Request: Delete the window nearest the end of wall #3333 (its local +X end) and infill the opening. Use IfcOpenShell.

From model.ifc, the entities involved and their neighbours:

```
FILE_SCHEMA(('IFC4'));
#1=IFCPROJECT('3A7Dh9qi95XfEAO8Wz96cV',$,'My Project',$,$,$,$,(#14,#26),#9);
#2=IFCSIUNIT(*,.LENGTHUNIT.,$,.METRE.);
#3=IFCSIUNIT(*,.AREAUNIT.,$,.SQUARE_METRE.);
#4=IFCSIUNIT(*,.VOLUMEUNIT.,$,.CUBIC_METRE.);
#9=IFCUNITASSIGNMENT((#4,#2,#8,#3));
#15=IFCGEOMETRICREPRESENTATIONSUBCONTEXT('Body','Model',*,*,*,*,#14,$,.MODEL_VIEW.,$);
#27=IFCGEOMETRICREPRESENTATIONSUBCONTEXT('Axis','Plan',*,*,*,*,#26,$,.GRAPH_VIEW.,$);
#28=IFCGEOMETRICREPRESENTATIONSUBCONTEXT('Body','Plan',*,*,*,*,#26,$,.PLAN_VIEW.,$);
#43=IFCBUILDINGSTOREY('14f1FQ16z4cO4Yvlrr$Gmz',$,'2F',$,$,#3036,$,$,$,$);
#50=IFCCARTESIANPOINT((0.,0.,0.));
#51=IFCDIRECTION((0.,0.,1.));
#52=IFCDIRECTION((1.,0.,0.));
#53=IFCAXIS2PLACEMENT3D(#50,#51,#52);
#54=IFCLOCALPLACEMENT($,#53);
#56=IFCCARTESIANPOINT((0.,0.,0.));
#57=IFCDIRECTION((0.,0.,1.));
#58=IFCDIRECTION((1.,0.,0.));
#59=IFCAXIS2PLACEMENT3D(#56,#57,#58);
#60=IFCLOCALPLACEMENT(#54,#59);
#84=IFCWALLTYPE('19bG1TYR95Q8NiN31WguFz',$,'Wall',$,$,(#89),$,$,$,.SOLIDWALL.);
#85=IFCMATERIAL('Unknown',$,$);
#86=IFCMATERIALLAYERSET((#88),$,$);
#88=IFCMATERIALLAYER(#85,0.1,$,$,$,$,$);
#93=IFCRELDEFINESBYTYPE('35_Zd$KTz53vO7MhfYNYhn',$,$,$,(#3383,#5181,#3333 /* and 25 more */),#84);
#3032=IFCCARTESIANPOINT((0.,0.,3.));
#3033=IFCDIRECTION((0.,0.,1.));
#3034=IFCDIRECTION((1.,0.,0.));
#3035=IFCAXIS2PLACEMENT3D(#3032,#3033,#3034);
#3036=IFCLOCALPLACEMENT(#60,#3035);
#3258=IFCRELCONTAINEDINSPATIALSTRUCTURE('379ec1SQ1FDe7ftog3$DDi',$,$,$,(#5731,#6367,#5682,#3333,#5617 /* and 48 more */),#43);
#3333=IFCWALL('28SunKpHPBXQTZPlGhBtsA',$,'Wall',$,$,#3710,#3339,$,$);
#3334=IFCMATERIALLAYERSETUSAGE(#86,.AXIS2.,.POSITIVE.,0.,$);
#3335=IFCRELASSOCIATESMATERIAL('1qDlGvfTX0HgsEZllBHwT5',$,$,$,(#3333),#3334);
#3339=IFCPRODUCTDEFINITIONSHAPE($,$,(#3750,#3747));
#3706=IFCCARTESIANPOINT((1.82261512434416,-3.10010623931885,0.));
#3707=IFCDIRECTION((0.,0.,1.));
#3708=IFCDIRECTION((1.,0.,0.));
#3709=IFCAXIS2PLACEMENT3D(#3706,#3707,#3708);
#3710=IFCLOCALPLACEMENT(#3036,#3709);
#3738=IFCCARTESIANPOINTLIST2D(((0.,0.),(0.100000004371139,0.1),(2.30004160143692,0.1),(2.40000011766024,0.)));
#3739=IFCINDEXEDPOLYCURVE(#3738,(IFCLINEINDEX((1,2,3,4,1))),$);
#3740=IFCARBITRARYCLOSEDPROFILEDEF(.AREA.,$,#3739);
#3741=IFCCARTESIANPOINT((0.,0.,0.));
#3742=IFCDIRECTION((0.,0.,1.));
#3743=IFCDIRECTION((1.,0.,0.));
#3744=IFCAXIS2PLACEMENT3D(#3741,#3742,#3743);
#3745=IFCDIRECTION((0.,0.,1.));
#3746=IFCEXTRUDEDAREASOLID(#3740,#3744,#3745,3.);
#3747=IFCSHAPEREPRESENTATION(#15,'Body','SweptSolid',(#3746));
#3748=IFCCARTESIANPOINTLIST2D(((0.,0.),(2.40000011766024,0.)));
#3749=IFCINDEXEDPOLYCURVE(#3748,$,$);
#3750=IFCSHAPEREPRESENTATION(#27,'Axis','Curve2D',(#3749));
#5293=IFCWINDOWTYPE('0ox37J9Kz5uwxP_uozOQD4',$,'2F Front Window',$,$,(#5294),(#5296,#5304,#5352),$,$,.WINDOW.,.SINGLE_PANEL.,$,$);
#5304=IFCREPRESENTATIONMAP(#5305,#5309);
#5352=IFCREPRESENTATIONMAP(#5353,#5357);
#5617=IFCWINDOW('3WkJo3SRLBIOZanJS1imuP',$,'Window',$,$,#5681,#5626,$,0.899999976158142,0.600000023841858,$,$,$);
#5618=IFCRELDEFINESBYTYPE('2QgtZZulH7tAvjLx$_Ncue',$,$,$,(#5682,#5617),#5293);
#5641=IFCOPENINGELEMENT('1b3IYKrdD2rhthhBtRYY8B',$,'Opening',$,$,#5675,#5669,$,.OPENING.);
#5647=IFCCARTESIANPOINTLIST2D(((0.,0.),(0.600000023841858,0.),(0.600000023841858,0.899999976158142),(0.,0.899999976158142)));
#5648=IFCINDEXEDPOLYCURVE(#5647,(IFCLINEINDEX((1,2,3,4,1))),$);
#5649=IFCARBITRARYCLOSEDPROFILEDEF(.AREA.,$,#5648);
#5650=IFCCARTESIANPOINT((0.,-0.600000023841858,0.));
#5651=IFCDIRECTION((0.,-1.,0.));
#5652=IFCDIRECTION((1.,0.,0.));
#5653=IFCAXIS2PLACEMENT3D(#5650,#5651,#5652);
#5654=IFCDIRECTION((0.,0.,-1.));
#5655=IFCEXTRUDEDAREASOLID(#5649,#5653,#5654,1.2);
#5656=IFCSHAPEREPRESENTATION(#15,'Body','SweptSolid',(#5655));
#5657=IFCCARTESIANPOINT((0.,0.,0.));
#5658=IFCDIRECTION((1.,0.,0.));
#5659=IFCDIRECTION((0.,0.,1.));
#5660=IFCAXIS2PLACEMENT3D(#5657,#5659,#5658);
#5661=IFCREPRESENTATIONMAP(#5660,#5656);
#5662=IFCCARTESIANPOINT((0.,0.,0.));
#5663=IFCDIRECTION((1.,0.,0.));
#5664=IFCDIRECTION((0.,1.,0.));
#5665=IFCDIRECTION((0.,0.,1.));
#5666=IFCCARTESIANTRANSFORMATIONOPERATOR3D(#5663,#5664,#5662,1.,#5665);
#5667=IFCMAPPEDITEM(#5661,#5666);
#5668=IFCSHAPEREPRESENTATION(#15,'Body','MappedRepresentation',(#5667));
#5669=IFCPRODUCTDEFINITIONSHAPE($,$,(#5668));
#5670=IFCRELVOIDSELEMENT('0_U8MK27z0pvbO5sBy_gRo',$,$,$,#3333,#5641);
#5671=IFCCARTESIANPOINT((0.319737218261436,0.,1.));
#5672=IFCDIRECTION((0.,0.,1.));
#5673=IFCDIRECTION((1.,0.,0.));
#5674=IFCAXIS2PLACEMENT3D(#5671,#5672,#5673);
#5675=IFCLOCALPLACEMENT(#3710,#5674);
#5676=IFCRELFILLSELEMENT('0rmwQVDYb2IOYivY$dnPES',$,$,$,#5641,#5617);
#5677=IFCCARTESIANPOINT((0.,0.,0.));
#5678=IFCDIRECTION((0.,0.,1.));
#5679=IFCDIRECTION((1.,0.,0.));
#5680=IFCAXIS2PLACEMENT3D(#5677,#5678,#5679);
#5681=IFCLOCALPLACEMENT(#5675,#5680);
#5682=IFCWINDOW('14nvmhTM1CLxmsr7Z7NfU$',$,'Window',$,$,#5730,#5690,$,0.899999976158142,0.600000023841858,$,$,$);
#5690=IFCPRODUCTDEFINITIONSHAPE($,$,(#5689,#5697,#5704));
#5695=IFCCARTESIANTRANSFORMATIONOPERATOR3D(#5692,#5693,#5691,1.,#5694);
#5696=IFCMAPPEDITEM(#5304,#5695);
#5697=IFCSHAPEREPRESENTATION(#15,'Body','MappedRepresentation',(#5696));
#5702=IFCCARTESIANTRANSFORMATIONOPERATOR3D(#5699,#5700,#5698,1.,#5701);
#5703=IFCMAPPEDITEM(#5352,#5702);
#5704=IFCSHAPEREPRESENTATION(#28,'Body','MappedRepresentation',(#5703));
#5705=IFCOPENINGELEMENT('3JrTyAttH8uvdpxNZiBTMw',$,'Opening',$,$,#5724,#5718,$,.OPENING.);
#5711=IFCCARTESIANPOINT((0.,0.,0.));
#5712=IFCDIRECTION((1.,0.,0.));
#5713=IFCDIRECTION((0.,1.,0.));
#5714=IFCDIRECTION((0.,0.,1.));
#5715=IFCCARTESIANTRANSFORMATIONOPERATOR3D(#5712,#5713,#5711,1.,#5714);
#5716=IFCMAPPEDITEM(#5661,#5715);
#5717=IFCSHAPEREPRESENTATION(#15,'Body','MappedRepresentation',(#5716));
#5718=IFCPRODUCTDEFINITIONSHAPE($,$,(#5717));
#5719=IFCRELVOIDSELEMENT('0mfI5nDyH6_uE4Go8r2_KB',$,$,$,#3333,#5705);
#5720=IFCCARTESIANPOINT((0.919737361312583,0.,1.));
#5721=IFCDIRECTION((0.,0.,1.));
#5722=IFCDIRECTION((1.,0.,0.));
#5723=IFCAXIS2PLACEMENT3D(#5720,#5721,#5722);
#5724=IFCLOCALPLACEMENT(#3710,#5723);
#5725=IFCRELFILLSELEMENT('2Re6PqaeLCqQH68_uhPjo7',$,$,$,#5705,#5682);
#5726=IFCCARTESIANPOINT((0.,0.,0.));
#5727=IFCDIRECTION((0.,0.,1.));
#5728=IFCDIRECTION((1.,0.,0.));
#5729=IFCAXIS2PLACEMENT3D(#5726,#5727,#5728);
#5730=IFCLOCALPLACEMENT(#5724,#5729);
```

```python
import ifcopenshell
import ifcopenshell.api.feature
import ifcopenshell.api.root
import ifcopenshell.geom
import ifcopenshell.util.shape

model = ifcopenshell.open("model.ifc")
settings = ifcopenshell.geom.settings()


def volume(element):
    """Net volume in cubic metres, openings subtracted."""
    shape = ifcopenshell.geom.create_shape(settings, element)
    return ifcopenshell.util.shape.get_volume(shape.geometry)


window = model.by_id(5682)
opening = window.FillsVoids[0].RelatingOpeningElement
wall = opening.VoidsElements[0].RelatingBuildingElement
before = volume(wall)

ifcopenshell.api.root.remove_product(model, product=window)
ifcopenshell.api.feature.remove_feature(model, feature=opening)

after = volume(wall)

print(f"wall volume {before:.3f} -> {after:.3f} m3")

model.write("model_v2.ifc")
```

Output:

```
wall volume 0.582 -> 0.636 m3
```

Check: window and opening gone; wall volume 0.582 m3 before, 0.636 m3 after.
